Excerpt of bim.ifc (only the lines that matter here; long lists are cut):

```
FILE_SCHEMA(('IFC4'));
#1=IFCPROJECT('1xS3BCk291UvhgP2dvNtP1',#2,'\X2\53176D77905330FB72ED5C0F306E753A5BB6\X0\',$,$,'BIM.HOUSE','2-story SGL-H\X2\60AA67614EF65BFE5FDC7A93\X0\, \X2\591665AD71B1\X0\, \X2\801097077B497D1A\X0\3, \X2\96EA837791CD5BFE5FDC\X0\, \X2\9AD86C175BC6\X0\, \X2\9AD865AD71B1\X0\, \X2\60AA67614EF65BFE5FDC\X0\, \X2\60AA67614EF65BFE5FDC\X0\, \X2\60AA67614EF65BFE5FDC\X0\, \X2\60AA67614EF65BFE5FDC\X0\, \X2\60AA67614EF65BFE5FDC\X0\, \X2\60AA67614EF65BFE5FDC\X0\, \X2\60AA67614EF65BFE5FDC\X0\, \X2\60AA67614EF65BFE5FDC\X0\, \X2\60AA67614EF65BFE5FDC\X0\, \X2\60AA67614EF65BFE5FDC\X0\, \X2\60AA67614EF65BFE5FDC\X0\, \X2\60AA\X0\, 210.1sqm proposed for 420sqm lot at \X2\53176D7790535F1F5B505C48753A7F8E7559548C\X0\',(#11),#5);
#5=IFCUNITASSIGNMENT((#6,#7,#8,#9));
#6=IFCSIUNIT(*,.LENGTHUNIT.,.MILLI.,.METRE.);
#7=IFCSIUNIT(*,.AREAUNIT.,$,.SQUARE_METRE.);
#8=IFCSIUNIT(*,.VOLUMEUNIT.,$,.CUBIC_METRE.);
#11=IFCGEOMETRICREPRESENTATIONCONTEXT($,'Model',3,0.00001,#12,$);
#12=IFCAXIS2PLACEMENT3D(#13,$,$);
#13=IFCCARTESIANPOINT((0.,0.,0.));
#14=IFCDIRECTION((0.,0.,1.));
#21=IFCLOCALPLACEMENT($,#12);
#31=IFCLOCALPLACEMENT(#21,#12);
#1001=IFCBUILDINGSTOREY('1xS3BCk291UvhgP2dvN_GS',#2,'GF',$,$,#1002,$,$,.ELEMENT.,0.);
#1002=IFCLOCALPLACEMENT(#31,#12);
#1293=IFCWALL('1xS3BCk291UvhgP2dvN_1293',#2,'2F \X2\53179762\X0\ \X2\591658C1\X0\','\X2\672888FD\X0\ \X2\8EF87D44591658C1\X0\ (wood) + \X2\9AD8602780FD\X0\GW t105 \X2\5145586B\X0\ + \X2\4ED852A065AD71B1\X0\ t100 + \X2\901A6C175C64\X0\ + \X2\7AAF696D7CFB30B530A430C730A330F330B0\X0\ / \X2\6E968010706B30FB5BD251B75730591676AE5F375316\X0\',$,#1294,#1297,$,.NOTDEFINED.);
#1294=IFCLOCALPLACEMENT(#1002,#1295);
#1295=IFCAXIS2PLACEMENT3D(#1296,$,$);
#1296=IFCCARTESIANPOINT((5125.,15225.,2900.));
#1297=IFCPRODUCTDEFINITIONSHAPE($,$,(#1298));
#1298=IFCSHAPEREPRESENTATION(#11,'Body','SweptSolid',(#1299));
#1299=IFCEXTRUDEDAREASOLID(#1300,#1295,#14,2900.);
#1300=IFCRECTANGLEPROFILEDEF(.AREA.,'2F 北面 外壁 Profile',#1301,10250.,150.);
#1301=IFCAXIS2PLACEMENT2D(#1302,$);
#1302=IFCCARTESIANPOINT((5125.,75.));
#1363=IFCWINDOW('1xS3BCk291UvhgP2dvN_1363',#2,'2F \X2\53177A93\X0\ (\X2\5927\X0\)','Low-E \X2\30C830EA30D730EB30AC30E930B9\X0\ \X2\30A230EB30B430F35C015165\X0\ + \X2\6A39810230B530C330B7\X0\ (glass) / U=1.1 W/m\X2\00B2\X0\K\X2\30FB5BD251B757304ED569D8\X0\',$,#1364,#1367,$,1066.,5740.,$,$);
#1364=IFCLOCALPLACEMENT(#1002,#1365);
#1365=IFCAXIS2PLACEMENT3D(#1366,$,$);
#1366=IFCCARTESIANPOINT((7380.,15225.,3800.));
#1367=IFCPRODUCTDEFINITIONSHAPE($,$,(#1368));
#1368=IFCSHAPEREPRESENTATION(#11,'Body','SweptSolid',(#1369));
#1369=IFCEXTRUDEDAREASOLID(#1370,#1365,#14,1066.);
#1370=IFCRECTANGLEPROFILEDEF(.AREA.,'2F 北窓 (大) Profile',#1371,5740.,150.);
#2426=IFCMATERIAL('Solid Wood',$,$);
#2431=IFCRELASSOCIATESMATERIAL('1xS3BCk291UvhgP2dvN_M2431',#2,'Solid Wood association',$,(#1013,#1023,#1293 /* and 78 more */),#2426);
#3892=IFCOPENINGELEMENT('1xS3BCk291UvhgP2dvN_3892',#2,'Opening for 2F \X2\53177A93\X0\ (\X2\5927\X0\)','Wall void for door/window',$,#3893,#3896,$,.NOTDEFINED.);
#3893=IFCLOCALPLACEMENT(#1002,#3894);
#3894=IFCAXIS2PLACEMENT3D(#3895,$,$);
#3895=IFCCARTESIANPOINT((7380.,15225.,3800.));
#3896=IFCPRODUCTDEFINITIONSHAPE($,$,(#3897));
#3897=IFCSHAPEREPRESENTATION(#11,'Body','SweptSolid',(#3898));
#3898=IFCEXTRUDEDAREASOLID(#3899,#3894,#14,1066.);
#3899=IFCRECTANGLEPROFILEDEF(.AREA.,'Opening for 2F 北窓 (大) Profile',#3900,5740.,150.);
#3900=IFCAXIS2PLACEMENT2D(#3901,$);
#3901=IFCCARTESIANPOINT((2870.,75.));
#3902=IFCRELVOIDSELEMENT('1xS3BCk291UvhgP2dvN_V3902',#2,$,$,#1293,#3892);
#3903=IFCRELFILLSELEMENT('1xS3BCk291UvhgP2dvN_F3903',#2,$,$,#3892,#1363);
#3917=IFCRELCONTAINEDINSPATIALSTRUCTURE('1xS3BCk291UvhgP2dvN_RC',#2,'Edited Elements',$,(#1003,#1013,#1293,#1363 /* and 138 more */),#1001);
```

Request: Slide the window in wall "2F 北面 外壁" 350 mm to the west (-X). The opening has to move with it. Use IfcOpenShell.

```python
import ifcopenshell
import ifcopenshell.api.geometry
import ifcopenshell.util.placement
import ifcopenshell.util.unit

model = ifcopenshell.open("bim.ifc")
unit_scale = ifcopenshell.util.unit.calculate_unit_scale(model)

window = model.by_id(1363)
opening = window.FillsVoids[0].RelatingOpeningElement
wall = opening.VoidsElements[0].RelatingBuildingElement

wall_matrix = ifcopenshell.util.placement.get_local_placement(wall.ObjectPlacement)
shift = wall_matrix[:3, 0] * -0.35 / unit_scale
before = ifcopenshell.util.placement.get_local_placement(window.ObjectPlacement)[:3, 3].copy()

# The window is not placed relative to its opening, so move both.
for product in (opening, window):
    matrix = ifcopenshell.util.placement.get_local_placement(product.ObjectPlacement)
    matrix[:3, 3] += shift
    ifcopenshell.api.geometry.edit_object_placement(model, product=product, matrix=matrix, is_si=False)

after = ifcopenshell.util.placement.get_local_placement(window.ObjectPlacement)[:3, 3]
print("window moved by", (after - before).round(3) + 0.0)

model.write("bim_edited.ifc")
```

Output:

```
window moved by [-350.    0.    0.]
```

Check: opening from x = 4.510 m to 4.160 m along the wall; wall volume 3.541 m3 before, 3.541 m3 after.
